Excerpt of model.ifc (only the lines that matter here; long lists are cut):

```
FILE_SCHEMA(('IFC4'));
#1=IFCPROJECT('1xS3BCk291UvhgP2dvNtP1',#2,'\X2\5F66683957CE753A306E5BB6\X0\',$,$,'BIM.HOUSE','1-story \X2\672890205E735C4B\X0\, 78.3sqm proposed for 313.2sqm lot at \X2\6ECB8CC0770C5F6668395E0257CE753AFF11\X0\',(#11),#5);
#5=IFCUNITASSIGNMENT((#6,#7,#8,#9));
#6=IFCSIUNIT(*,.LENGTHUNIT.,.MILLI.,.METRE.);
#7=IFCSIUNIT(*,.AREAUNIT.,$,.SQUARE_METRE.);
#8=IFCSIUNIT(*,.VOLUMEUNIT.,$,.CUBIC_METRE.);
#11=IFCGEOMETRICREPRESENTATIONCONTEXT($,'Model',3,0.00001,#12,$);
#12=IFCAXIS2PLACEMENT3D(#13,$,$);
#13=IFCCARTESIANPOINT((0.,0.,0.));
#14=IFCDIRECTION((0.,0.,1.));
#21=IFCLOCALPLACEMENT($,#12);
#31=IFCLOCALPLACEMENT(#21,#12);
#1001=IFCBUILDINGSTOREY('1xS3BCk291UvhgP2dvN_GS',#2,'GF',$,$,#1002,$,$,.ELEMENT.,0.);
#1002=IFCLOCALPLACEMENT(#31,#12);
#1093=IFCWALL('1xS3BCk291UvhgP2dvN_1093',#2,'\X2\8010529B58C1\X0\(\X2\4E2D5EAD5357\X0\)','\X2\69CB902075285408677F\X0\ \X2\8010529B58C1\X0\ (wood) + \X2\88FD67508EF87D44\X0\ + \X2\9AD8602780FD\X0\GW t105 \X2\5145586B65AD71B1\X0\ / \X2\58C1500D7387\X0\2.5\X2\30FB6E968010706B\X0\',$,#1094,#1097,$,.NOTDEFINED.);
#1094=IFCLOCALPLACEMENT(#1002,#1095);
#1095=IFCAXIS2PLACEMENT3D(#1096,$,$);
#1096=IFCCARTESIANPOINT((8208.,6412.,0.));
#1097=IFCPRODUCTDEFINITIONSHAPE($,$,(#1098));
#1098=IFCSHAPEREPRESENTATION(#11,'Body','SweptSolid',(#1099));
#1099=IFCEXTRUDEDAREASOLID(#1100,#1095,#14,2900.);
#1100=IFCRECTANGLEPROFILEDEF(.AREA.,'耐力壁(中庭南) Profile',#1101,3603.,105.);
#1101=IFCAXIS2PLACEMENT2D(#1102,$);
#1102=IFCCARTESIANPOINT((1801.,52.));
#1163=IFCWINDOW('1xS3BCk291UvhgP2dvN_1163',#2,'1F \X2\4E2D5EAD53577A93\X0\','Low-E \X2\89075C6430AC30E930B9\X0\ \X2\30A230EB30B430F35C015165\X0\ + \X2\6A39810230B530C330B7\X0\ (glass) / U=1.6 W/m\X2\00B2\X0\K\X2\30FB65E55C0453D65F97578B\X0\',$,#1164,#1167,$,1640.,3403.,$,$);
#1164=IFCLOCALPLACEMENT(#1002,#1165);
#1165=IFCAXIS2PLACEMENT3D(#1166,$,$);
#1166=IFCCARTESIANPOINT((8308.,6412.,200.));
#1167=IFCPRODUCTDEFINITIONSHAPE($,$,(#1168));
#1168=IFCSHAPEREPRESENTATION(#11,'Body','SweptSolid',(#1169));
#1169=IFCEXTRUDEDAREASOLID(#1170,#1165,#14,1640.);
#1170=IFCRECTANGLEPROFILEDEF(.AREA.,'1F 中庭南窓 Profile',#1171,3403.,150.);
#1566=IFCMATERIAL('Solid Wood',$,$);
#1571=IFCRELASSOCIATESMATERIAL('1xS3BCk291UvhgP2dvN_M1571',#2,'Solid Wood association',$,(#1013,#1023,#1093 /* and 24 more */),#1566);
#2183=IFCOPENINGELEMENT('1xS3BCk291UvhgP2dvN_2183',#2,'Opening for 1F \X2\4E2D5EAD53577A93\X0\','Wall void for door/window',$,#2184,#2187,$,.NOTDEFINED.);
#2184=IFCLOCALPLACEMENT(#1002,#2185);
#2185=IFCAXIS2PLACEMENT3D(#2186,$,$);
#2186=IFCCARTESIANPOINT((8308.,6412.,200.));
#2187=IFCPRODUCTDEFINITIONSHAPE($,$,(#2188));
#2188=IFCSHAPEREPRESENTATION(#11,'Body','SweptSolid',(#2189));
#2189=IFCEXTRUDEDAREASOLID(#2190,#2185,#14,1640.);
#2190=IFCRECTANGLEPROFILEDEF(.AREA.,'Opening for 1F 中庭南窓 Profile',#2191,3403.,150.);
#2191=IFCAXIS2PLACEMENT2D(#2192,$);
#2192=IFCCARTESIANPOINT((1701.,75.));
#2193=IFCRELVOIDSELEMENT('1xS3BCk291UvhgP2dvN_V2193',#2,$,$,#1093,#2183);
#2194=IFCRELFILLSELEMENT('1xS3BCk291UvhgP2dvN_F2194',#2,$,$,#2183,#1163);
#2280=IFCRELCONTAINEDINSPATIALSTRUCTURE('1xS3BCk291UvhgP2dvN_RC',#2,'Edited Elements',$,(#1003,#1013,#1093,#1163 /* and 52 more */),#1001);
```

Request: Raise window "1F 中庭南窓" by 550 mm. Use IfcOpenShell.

```python
import numpy as np
import ifcopenshell
import ifcopenshell.api.geometry
import ifcopenshell.util.placement
import ifcopenshell.util.unit

model = ifcopenshell.open("model.ifc")
unit_scale = ifcopenshell.util.unit.calculate_unit_scale(model)

window = model.by_id(1163)
opening = window.FillsVoids[0].RelatingOpeningElement
dz = 0.55 / unit_scale

shift = np.array([0.0, 0.0, dz])
# The window is not placed relative to its opening, so move both.
for product in (opening, window):
    matrix = ifcopenshell.util.placement.get_local_placement(product.ObjectPlacement)
    matrix[:3, 3] += shift
    ifcopenshell.api.geometry.edit_object_placement(model, product=product, matrix=matrix, is_si=False)

print(f"moved by {dz * unit_scale:+.3f} m")

model.write("model_rev.ifc")
```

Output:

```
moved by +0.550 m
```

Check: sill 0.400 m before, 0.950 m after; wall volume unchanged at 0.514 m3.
